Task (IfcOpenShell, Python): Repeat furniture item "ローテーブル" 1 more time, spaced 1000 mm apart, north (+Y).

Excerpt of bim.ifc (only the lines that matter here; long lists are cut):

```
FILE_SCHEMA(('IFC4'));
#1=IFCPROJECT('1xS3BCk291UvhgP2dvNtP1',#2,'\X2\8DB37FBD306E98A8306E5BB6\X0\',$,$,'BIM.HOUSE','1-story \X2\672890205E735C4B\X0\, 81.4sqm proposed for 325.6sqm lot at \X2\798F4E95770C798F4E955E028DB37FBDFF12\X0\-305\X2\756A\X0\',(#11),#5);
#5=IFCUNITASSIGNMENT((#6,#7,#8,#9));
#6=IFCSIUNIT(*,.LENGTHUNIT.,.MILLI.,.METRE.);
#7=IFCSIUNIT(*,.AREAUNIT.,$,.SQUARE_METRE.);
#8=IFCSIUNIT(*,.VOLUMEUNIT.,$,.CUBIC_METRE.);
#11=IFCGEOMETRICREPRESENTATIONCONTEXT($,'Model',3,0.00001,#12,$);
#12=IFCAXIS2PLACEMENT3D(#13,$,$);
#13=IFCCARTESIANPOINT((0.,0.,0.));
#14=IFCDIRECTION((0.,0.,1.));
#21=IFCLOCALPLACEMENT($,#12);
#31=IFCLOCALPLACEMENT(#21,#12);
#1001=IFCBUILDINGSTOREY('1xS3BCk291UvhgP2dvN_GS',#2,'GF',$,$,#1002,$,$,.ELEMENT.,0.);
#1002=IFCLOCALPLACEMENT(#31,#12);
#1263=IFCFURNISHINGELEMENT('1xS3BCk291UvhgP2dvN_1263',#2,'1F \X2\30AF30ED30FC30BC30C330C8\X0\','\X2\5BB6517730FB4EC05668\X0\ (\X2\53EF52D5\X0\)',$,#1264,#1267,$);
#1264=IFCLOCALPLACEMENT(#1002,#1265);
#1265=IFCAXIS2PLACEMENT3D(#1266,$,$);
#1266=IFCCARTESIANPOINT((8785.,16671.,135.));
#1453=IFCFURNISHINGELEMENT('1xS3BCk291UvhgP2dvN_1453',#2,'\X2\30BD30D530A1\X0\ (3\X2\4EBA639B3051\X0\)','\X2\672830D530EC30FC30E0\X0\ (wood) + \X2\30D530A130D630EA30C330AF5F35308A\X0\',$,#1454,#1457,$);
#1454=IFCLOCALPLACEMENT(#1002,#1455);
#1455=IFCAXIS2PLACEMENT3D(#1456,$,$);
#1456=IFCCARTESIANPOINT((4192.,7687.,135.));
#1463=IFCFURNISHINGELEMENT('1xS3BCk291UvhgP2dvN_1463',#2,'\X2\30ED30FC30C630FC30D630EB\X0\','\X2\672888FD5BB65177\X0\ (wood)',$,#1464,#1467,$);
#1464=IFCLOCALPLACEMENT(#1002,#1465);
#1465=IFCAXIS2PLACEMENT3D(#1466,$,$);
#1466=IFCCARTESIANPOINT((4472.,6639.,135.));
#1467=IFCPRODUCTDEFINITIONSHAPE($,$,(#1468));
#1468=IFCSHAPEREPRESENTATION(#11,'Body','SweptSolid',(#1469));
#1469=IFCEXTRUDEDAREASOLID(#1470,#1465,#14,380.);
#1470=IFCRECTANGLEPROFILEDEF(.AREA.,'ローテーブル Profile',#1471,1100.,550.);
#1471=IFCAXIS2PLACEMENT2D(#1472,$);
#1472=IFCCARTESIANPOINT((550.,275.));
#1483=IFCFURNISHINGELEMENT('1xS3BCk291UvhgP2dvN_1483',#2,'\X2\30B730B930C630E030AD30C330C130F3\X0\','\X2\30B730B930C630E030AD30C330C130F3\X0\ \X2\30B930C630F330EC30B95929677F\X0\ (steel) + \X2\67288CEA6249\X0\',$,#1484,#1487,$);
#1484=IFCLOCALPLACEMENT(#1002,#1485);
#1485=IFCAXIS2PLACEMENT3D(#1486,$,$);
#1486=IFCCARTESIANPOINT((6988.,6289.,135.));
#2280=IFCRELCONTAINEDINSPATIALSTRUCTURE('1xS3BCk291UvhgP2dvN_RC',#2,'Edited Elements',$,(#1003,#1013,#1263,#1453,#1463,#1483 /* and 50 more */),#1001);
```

```python
import numpy as np
import ifcopenshell
import ifcopenshell.api.geometry
import ifcopenshell.api.root
import ifcopenshell.util.element
import ifcopenshell.util.placement

model = ifcopenshell.open("bim.ifc")


def reuse_history(source, copy):
    """copy_class also copies each property set's owner history, people and application; keep the originals."""
    for rel in copy.IsDefinedBy:
        if rel.is_a("IfcRelDefinesByProperties") and (history := rel.RelatingPropertyDefinition.OwnerHistory):
            rel.RelatingPropertyDefinition.OwnerHistory = source.OwnerHistory
            ifcopenshell.util.element.remove_deep2(model, history)


source = model.by_guid("1xS3BCk291UvhgP2dvN_1463")
base = ifcopenshell.util.placement.get_local_placement(source.ObjectPlacement)
step = np.array([0.0, 1.0, 0.0]) * 1000.0

for i in range(1, 2):
    copy = ifcopenshell.api.root.copy_class(model, product=source)
    copy.Representation = ifcopenshell.util.element.copy_deep(
        model, source.Representation, exclude=["IfcGeometricRepresentationContext", "IfcRepresentationMap"]
    )
    reuse_history(source, copy)
    matrix = base.copy()
    matrix[:3, 3] += i * step
    print("added at", matrix[:3, 3].round(3) + 0.0)
    ifcopenshell.api.geometry.edit_object_placement(model, product=copy, matrix=matrix, is_si=False)

model.write("bim_v2.ifc")
```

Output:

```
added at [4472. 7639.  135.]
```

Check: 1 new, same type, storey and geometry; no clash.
